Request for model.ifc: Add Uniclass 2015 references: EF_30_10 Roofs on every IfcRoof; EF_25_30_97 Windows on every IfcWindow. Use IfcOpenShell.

First a look at what the model holds.

```python
import ifcopenshell

model = ifcopenshell.open("model.ifc")
print(model.schema)
print("classifications:", [c.Name for c in model.by_type("IfcClassification")])
for ifc_class in ("IfcDoor", "IfcRoof", "IfcStair", "IfcWall", "IfcWindow"):
    print(ifc_class, len(model.by_type(ifc_class)))
```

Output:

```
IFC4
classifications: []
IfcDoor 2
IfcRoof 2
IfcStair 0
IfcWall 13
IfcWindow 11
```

```python
import ifcopenshell
import ifcopenshell.api.classification

model = ifcopenshell.open("model.ifc")

system = ifcopenshell.api.classification.add_classification(model, classification="Uniclass 2015")

codes = {
    "IfcRoof": ("EF_30_10", "Roofs"),
    "IfcWindow": ("EF_25_30_97", "Windows"),
}
for ifc_class, (code, name) in codes.items():
    products = model.by_type(ifc_class)
    ifcopenshell.api.classification.add_reference(
        model, products=products, classification=system, identification=code, name=name
    )
    print(code, len(products))

model.write("model_edited.ifc")
```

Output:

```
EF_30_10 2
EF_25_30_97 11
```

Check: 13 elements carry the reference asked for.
